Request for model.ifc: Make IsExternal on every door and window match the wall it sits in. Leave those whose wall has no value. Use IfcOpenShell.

First a look at what the model holds.

```python
import ifcopenshell
import ifcopenshell.util.element

model = ifcopenshell.open("model.ifc")
print(model.schema)
seen = {}
for e in model.by_type("IfcDoor") + model.by_type("IfcWindow"):
    if not e.FillsVoids:
        continue
    host = e.FillsVoids[0].RelatingOpeningElement.VoidsElements[0].RelatingBuildingElement
    own = ifcopenshell.util.element.get_pset(e, f"Pset_{e.is_a()[3:].removesuffix('StandardCase')}Common", "IsExternal")
    wall = ifcopenshell.util.element.get_pset(host, "Pset_WallCommon", "IsExternal")
    seen[e.is_a(), own, wall] = seen.get((e.is_a(), own, wall), 0) + 1
for (cls, own, wall), count in sorted(seen.items(), key=str):
    print(count, cls, "IsExternal:", own, "| host wall:", wall)
```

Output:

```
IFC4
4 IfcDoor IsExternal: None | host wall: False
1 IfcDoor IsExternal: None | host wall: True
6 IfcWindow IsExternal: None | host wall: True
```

```python
import ifcopenshell
import ifcopenshell.api.pset
import ifcopenshell.util.element

model = ifcopenshell.open("model.ifc")

count = 0
for ifc_class, pset_name in (("IfcDoor", "Pset_DoorCommon"), ("IfcWindow", "Pset_WindowCommon")):
    for e in model.by_type(ifc_class):
        if not e.FillsVoids:
            continue
        host = e.FillsVoids[0].RelatingOpeningElement.VoidsElements[0].RelatingBuildingElement
        external = ifcopenshell.util.element.get_pset(host, "Pset_WallCommon", "IsExternal")
        if external is None or ifcopenshell.util.element.get_pset(e, pset_name, "IsExternal") == external:
            continue
        pset = ifcopenshell.api.pset.add_pset(model, product=e, name=pset_name)
        ifcopenshell.api.pset.edit_pset(model, pset=pset, properties={"IsExternal": external})
        count += 1

print(count, "updated")

model.write("model_rev.ifc")
```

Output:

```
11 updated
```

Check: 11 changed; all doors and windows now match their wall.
